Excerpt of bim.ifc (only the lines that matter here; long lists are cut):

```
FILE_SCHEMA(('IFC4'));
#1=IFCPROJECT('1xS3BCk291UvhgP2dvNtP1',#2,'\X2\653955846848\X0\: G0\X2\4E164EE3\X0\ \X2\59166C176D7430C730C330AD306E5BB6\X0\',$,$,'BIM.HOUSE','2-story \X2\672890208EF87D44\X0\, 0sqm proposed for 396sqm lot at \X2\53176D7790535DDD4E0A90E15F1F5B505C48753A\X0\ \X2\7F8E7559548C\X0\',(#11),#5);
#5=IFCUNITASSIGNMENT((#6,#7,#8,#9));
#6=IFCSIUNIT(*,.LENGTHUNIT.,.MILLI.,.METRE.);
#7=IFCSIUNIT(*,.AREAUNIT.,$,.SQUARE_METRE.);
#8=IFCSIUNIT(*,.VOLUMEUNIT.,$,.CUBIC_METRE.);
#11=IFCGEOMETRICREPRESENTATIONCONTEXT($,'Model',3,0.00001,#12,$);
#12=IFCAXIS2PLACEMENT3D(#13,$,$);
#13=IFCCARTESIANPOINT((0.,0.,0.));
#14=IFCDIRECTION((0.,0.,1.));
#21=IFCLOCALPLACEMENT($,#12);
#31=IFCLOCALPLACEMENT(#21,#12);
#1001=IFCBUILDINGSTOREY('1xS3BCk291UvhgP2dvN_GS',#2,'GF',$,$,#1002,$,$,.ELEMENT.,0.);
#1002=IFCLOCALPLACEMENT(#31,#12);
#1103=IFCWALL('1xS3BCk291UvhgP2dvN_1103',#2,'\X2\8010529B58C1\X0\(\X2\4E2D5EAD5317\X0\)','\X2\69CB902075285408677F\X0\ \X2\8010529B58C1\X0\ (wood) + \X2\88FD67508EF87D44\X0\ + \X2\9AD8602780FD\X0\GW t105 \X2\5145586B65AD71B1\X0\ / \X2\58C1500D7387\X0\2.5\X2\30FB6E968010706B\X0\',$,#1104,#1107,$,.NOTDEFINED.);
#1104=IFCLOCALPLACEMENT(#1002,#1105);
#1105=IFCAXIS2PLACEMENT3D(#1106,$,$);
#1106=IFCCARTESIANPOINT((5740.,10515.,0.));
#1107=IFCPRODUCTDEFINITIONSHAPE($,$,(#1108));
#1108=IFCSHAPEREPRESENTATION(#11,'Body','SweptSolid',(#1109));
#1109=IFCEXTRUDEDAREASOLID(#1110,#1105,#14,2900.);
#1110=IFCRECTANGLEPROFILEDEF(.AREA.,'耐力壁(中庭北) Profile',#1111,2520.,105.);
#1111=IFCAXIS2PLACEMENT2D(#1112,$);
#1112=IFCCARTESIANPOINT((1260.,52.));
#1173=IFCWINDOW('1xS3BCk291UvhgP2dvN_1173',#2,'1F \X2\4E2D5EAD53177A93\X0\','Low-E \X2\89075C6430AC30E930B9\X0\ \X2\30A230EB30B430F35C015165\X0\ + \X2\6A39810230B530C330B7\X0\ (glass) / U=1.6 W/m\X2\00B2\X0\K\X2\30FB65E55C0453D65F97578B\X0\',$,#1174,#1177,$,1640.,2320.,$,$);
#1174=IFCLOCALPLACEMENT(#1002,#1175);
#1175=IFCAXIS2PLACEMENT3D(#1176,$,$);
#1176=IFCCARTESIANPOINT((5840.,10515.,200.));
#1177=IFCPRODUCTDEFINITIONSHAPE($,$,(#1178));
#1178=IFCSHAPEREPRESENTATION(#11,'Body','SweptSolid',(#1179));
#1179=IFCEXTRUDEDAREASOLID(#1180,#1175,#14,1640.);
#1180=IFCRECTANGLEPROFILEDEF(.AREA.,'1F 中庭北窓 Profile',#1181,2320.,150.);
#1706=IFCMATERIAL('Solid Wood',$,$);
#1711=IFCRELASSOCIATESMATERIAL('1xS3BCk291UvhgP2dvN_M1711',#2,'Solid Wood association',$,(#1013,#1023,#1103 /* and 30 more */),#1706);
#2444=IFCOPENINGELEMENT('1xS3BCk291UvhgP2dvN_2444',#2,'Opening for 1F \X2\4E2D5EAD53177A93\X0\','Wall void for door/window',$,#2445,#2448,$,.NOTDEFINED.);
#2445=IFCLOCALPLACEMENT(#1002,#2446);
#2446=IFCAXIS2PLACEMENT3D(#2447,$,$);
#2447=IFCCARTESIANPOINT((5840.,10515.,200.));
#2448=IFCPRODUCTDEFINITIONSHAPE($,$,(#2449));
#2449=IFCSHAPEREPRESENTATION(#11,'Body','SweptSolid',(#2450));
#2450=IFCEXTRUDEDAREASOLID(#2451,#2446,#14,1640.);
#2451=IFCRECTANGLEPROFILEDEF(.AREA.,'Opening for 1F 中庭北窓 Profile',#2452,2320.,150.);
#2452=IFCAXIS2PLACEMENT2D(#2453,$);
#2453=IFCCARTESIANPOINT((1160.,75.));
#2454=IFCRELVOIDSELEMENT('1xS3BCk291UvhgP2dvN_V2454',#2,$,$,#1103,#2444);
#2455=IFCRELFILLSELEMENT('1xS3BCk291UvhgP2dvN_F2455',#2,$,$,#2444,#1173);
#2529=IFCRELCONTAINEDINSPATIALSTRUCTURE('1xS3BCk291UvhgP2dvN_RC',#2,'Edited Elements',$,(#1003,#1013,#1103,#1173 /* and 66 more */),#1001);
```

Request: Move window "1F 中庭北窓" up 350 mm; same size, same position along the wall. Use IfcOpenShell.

```python
import numpy as np
import ifcopenshell
import ifcopenshell.api.geometry
import ifcopenshell.util.placement
import ifcopenshell.util.unit

model = ifcopenshell.open("bim.ifc")
unit_scale = ifcopenshell.util.unit.calculate_unit_scale(model)

window = model.by_guid("1xS3BCk291UvhgP2dvN_1173")
opening = window.FillsVoids[0].RelatingOpeningElement
dz = 0.35 / unit_scale

shift = np.array([0.0, 0.0, dz])
# The window is not placed relative to its opening, so move both.
for product in (opening, window):
    matrix = ifcopenshell.util.placement.get_local_placement(product.ObjectPlacement)
    matrix[:3, 3] += shift
    ifcopenshell.api.geometry.edit_object_placement(model, product=product, matrix=matrix, is_si=False)

print(f"moved by {dz * unit_scale:+.3f} m")

model.write("bim_updated.ifc")
```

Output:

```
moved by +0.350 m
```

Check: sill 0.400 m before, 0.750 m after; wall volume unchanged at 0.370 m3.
